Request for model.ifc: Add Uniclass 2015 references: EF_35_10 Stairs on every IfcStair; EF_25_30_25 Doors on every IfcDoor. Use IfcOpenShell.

First a look at what the model holds.

```python
import ifcopenshell

model = ifcopenshell.open("model.ifc")
print(model.schema)
print("classifications:", [c.Name for c in model.by_type("IfcClassification")])
for ifc_class in ("IfcDoor", "IfcRoof", "IfcStair", "IfcWall", "IfcWindow"):
    print(ifc_class, len(model.by_type(ifc_class)))
```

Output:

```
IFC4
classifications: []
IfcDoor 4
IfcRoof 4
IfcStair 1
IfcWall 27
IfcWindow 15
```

```python
import ifcopenshell
import ifcopenshell.api.classification

model = ifcopenshell.open("model.ifc")

system = ifcopenshell.api.classification.add_classification(model, classification="Uniclass 2015")

codes = {
    "IfcStair": ("EF_35_10", "Stairs"),
    "IfcDoor": ("EF_25_30_25", "Doors"),
}
for ifc_class, (code, name) in codes.items():
    products = model.by_type(ifc_class)
    ifcopenshell.api.classification.add_reference(
        model, products=products, classification=system, identification=code, name=name
    )
    print(code, len(products))

model.write("model_updated.ifc")
```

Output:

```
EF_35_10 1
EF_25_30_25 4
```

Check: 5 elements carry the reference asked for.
